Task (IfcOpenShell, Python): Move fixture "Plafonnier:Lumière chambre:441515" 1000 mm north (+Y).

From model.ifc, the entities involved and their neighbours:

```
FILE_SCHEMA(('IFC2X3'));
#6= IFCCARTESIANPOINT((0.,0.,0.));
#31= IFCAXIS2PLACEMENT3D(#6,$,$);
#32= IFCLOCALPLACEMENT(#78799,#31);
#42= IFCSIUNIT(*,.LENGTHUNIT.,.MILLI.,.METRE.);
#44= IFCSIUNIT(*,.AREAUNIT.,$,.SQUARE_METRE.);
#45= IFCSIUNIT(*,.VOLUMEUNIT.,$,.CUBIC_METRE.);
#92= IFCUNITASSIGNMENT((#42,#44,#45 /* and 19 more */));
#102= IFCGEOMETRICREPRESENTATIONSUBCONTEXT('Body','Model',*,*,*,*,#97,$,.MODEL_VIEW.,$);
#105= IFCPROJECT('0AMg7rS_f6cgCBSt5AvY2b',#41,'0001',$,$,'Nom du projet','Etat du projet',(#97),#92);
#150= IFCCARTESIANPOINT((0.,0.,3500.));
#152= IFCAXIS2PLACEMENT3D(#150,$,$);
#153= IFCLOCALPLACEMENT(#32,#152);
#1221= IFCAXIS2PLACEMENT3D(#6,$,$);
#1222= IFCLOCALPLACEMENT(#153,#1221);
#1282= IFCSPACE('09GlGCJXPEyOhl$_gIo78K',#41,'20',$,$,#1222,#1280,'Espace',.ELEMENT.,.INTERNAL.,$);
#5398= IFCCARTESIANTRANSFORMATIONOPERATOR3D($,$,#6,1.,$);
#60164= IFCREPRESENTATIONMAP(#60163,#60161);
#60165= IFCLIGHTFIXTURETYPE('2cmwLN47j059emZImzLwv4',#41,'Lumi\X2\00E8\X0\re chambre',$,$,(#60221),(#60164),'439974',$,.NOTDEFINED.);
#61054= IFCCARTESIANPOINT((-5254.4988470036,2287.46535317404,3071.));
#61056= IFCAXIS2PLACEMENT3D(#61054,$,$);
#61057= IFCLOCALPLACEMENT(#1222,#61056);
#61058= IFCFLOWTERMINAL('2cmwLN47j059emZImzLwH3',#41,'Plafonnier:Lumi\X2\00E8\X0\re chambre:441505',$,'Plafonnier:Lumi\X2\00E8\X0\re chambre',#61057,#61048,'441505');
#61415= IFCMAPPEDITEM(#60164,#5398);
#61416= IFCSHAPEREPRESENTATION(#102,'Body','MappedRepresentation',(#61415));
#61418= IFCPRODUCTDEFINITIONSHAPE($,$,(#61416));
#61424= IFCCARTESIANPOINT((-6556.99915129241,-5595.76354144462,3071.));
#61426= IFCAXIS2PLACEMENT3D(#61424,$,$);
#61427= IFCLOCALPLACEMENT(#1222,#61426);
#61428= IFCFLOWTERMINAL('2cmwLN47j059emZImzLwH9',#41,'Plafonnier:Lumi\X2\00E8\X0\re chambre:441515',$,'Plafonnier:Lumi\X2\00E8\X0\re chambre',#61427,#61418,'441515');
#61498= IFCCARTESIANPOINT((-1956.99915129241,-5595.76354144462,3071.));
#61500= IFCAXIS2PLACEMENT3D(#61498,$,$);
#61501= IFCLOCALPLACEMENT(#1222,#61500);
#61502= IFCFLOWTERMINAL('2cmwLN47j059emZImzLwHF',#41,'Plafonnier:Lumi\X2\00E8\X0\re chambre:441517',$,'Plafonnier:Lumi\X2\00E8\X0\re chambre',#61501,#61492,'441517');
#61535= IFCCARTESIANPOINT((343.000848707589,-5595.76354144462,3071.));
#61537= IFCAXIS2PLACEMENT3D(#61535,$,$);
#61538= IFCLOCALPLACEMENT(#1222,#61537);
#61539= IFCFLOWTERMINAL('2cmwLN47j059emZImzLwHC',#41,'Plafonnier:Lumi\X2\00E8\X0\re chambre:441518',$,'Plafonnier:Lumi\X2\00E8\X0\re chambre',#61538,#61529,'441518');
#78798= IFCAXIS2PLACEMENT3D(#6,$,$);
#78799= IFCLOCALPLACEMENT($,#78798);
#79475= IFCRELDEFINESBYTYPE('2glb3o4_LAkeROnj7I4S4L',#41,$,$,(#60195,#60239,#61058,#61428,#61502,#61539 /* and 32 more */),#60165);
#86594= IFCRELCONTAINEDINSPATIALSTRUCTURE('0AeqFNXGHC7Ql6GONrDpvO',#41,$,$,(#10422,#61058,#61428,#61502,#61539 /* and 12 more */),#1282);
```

```python
import ifcopenshell
import ifcopenshell.api.geometry
import ifcopenshell.util.placement
import ifcopenshell.util.unit

model = ifcopenshell.open("model.ifc")
unit_scale = ifcopenshell.util.unit.calculate_unit_scale(model)

item = model.by_id(61428)
matrix = ifcopenshell.util.placement.get_local_placement(item.ObjectPlacement)
matrix[1, 3] += 1 / unit_scale
ifcopenshell.api.geometry.edit_object_placement(model, product=item, matrix=matrix, is_si=False)

print(ifcopenshell.util.placement.get_local_placement(item.ObjectPlacement).round(3) + 0.0)

model.write("model_edited.ifc")
```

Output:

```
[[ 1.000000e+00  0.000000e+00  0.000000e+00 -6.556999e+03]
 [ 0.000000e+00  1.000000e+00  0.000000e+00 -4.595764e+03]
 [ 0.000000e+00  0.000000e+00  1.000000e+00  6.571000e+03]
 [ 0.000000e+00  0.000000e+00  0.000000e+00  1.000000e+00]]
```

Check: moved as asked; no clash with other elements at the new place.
